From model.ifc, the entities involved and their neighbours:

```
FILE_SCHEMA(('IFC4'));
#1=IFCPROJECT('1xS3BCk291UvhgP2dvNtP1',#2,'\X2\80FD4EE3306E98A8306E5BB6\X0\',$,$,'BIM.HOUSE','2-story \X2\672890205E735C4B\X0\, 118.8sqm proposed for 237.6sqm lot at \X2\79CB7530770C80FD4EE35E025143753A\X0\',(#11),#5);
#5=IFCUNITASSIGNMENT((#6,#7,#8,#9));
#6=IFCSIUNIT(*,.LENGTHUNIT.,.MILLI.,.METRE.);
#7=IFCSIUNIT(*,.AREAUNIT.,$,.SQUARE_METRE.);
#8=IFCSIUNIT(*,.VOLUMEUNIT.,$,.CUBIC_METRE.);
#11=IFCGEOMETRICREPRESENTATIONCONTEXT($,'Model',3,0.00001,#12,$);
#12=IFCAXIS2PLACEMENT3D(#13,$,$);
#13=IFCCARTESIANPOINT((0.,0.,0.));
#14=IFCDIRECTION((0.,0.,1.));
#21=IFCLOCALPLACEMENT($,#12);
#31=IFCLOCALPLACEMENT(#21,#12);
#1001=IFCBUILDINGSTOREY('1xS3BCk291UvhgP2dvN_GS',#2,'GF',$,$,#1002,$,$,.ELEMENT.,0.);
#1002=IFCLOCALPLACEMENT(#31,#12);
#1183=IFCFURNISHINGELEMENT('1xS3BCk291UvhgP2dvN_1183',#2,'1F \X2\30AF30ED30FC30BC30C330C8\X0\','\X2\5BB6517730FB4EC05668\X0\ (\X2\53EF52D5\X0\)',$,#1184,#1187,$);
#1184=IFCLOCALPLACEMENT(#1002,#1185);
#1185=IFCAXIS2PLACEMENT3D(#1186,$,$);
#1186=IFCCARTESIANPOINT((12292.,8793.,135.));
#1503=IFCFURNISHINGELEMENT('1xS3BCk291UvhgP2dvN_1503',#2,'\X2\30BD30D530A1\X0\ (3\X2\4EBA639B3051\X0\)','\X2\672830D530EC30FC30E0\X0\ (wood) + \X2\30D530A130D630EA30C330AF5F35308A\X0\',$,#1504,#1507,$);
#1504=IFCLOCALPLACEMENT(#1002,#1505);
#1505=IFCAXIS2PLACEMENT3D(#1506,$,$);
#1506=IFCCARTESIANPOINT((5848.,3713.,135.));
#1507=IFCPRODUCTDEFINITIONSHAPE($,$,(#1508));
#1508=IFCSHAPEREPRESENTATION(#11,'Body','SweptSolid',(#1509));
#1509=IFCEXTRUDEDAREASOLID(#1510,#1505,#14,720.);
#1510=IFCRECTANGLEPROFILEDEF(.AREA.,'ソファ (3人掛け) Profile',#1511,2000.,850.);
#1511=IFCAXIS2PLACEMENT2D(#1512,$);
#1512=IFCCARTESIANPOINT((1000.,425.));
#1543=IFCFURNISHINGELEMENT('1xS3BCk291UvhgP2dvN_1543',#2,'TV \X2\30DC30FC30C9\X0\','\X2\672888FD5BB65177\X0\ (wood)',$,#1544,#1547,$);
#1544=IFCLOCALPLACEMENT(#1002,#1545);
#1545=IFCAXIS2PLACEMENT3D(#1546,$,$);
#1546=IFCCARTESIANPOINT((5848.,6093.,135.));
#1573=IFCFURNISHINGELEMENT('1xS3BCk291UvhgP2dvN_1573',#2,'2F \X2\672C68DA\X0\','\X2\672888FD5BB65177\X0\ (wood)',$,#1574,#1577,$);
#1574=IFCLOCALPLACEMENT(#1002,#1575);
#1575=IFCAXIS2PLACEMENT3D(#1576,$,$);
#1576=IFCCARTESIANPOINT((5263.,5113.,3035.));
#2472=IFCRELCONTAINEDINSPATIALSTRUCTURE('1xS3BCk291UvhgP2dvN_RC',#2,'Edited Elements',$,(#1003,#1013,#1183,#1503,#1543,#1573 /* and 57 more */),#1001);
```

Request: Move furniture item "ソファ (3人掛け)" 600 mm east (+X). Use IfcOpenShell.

```python
import ifcopenshell
import ifcopenshell.api.geometry
import ifcopenshell.util.placement
import ifcopenshell.util.unit

model = ifcopenshell.open("model.ifc")
unit_scale = ifcopenshell.util.unit.calculate_unit_scale(model)

item = model.by_id(1503)
matrix = ifcopenshell.util.placement.get_local_placement(item.ObjectPlacement)
matrix[0, 3] += 0.6 / unit_scale
ifcopenshell.api.geometry.edit_object_placement(model, product=item, matrix=matrix, is_si=False)

print(ifcopenshell.util.placement.get_local_placement(item.ObjectPlacement).round(3) + 0.0)

model.write("model_edited.ifc")
```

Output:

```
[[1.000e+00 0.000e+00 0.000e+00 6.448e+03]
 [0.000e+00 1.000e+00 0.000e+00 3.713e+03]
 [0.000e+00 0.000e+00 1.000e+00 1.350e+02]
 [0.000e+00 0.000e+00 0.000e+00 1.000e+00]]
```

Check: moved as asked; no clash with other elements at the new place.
